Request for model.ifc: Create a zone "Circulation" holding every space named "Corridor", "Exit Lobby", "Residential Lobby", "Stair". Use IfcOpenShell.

First a look at what the model holds.

```python
import ifcopenshell

model = ifcopenshell.open("model.ifc")
print(model.schema)
seen = {}
for space in model.by_type("IfcSpace"):
    seen[space.LongName] = seen.get(space.LongName, 0) + 1
for name, count in sorted(seen.items(), key=str):
    print(count, "x", name)
print("zones:", [z.Name for z in model.by_type("IfcZone")][:20])
```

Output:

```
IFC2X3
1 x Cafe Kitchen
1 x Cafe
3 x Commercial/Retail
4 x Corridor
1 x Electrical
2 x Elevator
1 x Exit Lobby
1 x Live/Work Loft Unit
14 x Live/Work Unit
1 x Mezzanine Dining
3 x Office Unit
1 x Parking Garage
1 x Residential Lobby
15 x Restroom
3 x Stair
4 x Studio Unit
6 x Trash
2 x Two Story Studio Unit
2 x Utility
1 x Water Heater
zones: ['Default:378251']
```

```python
import ifcopenshell
import ifcopenshell.api.group
import ifcopenshell.api.root

model = ifcopenshell.open("model.ifc")

names = {"Corridor", "Exit Lobby", "Residential Lobby", "Stair"}
spaces = [s for s in model.by_type("IfcSpace") if s.LongName in names]

zone = ifcopenshell.api.root.create_entity(model, ifc_class="IfcZone", name="Circulation")
ifcopenshell.api.group.assign_group(model, products=spaces, group=zone)
print(len(spaces), "spaces in", zone.Name)

model.write("model-out.ifc")
```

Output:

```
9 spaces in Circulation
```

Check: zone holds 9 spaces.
